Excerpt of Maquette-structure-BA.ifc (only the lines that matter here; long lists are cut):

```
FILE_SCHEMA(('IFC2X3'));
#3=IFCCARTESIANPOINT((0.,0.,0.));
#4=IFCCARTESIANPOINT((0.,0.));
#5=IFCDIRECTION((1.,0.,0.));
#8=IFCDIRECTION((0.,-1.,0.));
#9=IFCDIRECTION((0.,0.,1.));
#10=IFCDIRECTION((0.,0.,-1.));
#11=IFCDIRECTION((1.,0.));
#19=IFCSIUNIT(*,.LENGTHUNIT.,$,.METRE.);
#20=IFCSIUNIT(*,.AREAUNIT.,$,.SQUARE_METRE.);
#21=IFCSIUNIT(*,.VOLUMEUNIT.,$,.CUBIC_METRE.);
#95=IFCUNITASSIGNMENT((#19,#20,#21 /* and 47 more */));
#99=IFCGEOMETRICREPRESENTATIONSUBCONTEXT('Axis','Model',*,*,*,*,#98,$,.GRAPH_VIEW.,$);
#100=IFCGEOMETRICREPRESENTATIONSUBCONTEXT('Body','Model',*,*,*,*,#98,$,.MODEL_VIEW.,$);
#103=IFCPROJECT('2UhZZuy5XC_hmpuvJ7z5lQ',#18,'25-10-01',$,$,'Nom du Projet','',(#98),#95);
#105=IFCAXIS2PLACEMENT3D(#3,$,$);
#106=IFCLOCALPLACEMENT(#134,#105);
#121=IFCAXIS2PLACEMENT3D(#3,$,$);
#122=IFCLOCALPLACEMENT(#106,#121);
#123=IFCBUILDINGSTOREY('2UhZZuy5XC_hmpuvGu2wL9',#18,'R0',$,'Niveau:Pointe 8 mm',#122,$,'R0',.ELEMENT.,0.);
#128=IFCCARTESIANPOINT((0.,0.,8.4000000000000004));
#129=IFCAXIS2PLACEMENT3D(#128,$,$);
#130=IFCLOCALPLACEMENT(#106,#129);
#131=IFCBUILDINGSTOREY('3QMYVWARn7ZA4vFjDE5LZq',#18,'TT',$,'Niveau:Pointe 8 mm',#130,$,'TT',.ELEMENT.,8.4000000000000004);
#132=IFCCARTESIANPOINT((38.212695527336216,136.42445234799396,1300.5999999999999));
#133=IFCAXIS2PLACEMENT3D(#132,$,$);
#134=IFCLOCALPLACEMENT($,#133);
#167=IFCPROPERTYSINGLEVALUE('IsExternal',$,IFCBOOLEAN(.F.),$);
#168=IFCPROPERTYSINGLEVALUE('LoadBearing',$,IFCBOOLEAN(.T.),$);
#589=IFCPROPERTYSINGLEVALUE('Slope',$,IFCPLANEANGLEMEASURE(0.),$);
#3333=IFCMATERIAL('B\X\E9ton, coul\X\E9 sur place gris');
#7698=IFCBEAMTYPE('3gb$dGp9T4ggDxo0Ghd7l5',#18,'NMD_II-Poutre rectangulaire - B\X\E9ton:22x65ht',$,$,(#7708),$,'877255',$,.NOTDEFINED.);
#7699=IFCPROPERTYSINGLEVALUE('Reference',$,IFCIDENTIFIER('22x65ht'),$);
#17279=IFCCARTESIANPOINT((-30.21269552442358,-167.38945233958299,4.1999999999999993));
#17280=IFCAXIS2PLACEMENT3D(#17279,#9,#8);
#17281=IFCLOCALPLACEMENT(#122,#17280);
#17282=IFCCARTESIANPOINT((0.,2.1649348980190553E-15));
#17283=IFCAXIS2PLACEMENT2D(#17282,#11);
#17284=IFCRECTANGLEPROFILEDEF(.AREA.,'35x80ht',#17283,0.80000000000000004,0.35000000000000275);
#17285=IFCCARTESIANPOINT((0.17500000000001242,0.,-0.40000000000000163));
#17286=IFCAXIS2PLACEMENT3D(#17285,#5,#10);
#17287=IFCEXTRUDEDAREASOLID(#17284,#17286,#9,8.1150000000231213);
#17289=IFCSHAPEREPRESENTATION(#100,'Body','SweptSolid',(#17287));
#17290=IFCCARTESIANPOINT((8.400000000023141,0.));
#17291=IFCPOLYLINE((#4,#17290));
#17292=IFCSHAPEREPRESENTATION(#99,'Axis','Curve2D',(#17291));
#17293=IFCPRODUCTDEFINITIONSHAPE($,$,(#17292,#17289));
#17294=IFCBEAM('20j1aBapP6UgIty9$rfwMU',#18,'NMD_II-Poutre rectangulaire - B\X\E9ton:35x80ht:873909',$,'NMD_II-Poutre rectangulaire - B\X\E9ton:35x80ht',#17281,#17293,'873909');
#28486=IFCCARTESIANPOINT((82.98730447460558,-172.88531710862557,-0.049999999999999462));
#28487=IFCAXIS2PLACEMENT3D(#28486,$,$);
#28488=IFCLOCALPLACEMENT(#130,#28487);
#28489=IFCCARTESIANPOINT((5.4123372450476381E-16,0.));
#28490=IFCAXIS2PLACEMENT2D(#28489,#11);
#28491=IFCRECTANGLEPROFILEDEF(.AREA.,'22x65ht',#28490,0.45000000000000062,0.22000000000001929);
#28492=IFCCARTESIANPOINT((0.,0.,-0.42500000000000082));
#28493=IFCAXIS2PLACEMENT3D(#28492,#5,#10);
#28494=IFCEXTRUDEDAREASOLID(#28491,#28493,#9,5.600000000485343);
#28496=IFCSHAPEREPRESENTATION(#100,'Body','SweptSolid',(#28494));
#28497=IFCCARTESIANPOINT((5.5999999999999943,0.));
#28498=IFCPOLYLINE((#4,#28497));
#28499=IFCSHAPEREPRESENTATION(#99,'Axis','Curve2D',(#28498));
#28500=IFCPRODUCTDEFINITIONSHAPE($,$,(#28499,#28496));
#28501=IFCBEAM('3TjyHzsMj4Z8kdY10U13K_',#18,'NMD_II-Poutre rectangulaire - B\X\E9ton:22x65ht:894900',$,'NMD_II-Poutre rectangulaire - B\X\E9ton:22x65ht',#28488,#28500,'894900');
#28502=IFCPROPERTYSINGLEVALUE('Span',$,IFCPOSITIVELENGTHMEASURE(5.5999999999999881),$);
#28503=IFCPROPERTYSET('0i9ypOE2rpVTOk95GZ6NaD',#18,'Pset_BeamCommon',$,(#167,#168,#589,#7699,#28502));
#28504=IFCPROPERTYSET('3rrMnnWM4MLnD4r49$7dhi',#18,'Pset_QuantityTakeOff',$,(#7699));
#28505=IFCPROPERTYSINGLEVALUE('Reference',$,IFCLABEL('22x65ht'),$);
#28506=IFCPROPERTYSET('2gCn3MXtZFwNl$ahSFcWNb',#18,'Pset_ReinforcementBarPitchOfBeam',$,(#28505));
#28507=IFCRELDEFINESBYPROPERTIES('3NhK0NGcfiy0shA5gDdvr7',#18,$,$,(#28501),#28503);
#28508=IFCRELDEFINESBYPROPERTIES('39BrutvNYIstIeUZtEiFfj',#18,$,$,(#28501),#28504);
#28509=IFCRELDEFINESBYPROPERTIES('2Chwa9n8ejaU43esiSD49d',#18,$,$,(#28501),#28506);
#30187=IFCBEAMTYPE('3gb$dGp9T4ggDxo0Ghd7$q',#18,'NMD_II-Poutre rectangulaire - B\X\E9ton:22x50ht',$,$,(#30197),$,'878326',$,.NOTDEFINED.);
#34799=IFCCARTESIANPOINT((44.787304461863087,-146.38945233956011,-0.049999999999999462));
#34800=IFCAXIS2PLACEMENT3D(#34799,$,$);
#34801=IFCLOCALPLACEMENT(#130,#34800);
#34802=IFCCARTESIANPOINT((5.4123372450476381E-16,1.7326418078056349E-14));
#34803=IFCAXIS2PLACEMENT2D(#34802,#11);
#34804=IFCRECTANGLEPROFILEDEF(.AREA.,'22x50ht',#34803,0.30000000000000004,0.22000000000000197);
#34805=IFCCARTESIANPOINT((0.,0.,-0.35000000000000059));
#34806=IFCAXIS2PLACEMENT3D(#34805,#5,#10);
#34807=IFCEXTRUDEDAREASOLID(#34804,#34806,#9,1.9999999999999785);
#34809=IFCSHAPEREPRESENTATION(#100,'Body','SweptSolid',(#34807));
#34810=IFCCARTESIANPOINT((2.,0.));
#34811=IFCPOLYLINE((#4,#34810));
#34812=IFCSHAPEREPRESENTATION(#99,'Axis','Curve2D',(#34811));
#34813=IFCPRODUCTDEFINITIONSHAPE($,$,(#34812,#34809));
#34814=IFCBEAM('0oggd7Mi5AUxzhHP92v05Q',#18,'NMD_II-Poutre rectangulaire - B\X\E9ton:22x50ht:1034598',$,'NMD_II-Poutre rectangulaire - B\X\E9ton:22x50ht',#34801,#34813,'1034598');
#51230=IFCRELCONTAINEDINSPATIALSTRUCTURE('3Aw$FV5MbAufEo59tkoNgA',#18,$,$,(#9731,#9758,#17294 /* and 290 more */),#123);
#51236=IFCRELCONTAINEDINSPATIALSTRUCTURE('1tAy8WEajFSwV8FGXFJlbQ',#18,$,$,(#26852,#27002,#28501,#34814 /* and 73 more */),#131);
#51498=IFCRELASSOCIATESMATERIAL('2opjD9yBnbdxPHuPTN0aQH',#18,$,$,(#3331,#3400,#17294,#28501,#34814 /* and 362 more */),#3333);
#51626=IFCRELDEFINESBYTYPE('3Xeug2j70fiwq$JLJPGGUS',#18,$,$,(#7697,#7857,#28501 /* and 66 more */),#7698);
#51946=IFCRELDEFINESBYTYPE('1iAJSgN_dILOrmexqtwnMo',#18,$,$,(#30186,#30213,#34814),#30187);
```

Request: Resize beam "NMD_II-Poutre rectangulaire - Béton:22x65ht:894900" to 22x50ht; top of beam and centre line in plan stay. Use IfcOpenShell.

```python
import ifcopenshell
import ifcopenshell.api.pset
import ifcopenshell.api.type
import ifcopenshell.util.element
import ifcopenshell.util.representation

model = ifcopenshell.open("Maquette-structure-BA.ifc")

member = model.by_guid("3TjyHzsMj4Z8kdY10U13K_")
source = next(p for p in model.by_type("IfcRectangleProfileDef") if p.ProfileName == "22x50ht")

body = ifcopenshell.util.representation.get_representation(member, "Model", "Body")
solid = body.Items[0]
old_profile = solid.SweptArea

# Copy the section's sizes but keep this member's own profile position.
profile = ifcopenshell.util.element.copy(model, source)
# Profiles are centred, so shift by half the change in depth to hold the top.
shift = (old_profile.XDim - profile.XDim) / 2
x, y = old_profile.Position.Location.Coordinates
up = (-1.0, 0.0)  # upwards, in the solid's own plane
location = model.createIfcCartesianPoint((x + up[0] * shift, y + up[1] * shift))
profile.Position = model.createIfcAxis2Placement2D(location, old_profile.Position.RefDirection)
solid.SweptArea = profile
if not model.get_total_inverses(old_profile):
    ifcopenshell.util.element.remove_deep2(model, old_profile)

new_type = model.by_id(30187)
ifcopenshell.api.type.assign_type(
    model, related_objects=[member], relating_type=new_type, should_map_representations=False
)
member.Name = member.Name.replace("22x65ht", "22x50ht")
member.ObjectType = "NMD_II-Poutre rectangulaire - Béton:22x50ht"
pset = model.by_id(ifcopenshell.util.element.get_pset(member, "Pset_BeamCommon", should_inherit=False)["id"])
ifcopenshell.api.pset.edit_pset(model, pset=pset, properties={"Reference": "22x50ht"})
pset = model.by_id(ifcopenshell.util.element.get_pset(member, "Pset_QuantityTakeOff", should_inherit=False)["id"])
ifcopenshell.api.pset.edit_pset(model, pset=pset, properties={"Reference": "22x50ht"})
pset = model.by_id(ifcopenshell.util.element.get_pset(member, "Pset_ReinforcementBarPitchOfBeam", should_inherit=False)["id"])
ifcopenshell.api.pset.edit_pset(model, pset=pset, properties={"Reference": "22x50ht"})

print(solid.SweptArea)

model.write("Maquette-structure-BA_v2.ifc")
```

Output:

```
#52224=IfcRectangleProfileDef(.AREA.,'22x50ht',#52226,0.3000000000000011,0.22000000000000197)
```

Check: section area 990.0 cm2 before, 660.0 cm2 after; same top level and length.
